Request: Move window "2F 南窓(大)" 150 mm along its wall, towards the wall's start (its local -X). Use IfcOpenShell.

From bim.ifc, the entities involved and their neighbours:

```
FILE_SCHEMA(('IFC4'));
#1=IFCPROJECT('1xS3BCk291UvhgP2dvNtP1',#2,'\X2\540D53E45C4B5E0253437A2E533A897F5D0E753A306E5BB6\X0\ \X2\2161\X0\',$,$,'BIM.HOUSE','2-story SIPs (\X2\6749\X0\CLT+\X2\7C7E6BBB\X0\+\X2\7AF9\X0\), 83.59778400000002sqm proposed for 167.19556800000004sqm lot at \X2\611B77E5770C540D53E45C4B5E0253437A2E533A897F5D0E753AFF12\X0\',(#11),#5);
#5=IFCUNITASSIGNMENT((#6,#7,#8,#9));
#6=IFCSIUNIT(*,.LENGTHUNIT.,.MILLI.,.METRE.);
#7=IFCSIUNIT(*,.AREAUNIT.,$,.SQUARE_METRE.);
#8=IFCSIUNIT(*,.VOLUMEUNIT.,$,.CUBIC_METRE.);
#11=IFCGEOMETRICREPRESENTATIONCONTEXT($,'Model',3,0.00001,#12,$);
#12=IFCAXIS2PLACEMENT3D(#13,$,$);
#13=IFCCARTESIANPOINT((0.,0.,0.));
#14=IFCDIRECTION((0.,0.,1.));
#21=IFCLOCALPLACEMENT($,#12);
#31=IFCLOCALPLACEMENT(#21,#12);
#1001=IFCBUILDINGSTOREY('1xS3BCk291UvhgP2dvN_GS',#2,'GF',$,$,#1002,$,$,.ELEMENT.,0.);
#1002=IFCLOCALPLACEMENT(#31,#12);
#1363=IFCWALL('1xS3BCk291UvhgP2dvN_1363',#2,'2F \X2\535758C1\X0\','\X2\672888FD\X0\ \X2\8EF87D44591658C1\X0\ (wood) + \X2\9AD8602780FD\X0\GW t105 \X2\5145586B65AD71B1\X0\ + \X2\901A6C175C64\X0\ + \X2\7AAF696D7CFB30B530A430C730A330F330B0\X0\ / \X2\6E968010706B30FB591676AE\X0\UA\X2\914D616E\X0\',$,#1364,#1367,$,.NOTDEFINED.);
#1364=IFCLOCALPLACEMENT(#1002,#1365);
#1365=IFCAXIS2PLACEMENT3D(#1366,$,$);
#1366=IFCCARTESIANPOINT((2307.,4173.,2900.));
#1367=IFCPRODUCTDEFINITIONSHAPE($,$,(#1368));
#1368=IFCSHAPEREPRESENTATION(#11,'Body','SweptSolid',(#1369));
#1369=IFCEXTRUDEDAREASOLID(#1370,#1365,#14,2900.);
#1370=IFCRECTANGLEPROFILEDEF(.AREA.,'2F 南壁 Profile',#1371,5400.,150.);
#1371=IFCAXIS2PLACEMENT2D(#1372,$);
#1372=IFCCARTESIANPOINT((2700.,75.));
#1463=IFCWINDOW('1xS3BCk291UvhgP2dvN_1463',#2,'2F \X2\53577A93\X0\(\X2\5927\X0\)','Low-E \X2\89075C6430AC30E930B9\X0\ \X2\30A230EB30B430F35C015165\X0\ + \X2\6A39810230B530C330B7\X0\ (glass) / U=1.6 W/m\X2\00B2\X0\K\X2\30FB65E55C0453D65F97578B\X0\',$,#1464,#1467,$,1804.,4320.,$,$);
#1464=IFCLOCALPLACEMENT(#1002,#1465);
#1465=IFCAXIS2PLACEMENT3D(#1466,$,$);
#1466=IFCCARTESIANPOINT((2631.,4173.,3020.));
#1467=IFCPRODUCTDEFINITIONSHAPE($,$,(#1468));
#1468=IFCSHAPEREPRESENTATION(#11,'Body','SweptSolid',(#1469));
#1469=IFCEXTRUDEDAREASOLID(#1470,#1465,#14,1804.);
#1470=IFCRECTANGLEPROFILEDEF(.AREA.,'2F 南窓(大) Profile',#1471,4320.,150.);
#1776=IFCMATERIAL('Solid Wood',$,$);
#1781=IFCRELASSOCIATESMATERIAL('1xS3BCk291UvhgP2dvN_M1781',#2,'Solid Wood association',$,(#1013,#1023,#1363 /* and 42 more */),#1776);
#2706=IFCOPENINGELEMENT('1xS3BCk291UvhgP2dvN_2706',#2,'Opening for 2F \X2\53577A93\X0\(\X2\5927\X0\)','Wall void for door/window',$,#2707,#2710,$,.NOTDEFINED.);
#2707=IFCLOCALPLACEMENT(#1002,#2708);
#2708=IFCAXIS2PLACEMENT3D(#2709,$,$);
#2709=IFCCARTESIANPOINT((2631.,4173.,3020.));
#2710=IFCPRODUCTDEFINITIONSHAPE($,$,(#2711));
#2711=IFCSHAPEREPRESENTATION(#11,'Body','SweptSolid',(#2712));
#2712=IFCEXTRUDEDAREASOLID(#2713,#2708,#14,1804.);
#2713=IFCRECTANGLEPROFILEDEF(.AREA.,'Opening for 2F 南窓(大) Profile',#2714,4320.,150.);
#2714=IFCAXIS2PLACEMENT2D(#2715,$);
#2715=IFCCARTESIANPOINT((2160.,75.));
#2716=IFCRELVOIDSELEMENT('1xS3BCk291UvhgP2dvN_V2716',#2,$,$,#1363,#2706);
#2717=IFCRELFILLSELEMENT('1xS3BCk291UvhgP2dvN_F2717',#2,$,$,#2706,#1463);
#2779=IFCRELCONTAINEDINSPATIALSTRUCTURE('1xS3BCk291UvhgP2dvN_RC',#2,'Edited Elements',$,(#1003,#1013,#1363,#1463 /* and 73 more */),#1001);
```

```python
import ifcopenshell
import ifcopenshell.api.geometry
import ifcopenshell.util.placement
import ifcopenshell.util.unit

model = ifcopenshell.open("bim.ifc")
unit_scale = ifcopenshell.util.unit.calculate_unit_scale(model)

window = model.by_guid("1xS3BCk291UvhgP2dvN_1463")
opening = window.FillsVoids[0].RelatingOpeningElement
wall = opening.VoidsElements[0].RelatingBuildingElement

wall_matrix = ifcopenshell.util.placement.get_local_placement(wall.ObjectPlacement)
shift = wall_matrix[:3, 0] * -0.15 / unit_scale
before = ifcopenshell.util.placement.get_local_placement(window.ObjectPlacement)[:3, 3].copy()

# The window is not placed relative to its opening, so move both.
for product in (opening, window):
    matrix = ifcopenshell.util.placement.get_local_placement(product.ObjectPlacement)
    matrix[:3, 3] += shift
    ifcopenshell.api.geometry.edit_object_placement(model, product=product, matrix=matrix, is_si=False)

after = ifcopenshell.util.placement.get_local_placement(window.ObjectPlacement)[:3, 3]
print("window moved by", (after - before).round(3) + 0.0)

model.write("bim_rev.ifc")
```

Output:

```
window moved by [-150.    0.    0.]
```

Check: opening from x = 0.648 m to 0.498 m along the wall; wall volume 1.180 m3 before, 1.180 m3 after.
